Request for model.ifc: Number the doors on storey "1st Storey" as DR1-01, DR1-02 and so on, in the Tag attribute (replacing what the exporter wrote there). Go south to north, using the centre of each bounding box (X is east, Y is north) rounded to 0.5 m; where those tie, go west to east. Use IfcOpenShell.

First a look at what the model holds.

```python
import ifcopenshell
import ifcopenshell.util.element
import ifcopenshell.util.placement

model = ifcopenshell.open("model.ifc")
print(model.schema)
storey = next(s for s in model.by_type("IfcBuildingStorey") if s.Name == "1st Storey")
doors = [e for e in ifcopenshell.util.element.get_decomposition(storey) if e.is_a("IfcDoor")]
for e in sorted(doors, key=lambda e: e.id()):
    origin = ifcopenshell.util.placement.get_local_placement(e.ObjectPlacement)[:3, 3]
    print(e.id(), e.Tag, e.Name, origin.round(2) + 0.0, sep=" | ")
```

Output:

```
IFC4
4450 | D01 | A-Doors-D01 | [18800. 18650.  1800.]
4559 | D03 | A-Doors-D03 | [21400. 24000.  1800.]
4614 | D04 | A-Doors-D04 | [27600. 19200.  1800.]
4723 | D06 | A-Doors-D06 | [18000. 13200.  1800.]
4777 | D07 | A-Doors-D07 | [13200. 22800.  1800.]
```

```python
import ifcopenshell
import ifcopenshell.geom
import ifcopenshell.util.element
import ifcopenshell.util.shape

model = ifcopenshell.open("model.ifc")
settings = ifcopenshell.geom.settings()
settings.set("use-world-coords", True)


def centre(element):
    shape = ifcopenshell.geom.create_shape(settings, element)
    return ifcopenshell.util.shape.get_bbox_centroid(shape.geometry)


storey = next(s for s in model.by_type("IfcBuildingStorey") if s.Name == "1st Storey")
doors = [e for e in ifcopenshell.util.element.get_decomposition(storey) if e.is_a("IfcDoor")]

# Insertion points can sit at a corner or the storey origin, so sort by the geometry (in metres).
centres = {e: centre(e) for e in doors}
doors.sort(key=lambda e: (round(centres[e][1] / 0.5), centres[e][0]))

for i, e in enumerate(doors, start=1):
    number = f"DR1-{i:02d}"
    e.Tag = number
    print(e.id(), number)

model.write("model_rev.ifc")
```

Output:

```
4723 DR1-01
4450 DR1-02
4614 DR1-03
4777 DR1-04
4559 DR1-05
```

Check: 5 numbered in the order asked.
